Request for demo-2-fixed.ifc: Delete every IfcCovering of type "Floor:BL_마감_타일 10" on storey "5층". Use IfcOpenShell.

First a look at what the model holds.

```python
import ifcopenshell
import ifcopenshell.util.element

model = ifcopenshell.open("demo-2-fixed.ifc")
print(model.schema)
storey = next(s for s in model.by_type("IfcBuildingStorey") if s.Name == "5층")
coverings = [e for e in ifcopenshell.util.element.get_decomposition(storey) if e.is_a("IfcCovering")]
seen = {}
for e in coverings:
    element_type = ifcopenshell.util.element.get_type(e)
    name = element_type.Name if element_type not in (None, e) else None
    seen[name] = seen.get(name, 0) + 1
for name, count in sorted(seen.items(), key=str):
    print(count, "x", name)
```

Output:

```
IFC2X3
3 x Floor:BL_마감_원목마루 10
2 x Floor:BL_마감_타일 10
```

```python
import ifcopenshell
import ifcopenshell.api.root
import ifcopenshell.util.element

model = ifcopenshell.open("demo-2-fixed.ifc")

storey = next(s for s in model.by_type("IfcBuildingStorey") if s.Name == "5층")
coverings = [e for e in ifcopenshell.util.element.get_decomposition(storey) if e.is_a("IfcCovering")]
targets = [e for e in coverings if (t := ifcopenshell.util.element.get_type(e)) not in (None, e) and t.Name == "Floor:BL_마감_타일 10"]

for e in targets:
    ifcopenshell.api.root.remove_product(model, product=e)
print(len(targets), "removed")

model.write("demo-2-fixed_edited.ifc")
```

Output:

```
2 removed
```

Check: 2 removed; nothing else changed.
